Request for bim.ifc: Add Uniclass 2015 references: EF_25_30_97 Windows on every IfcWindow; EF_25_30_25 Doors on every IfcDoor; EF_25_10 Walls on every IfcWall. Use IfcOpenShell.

First a look at what the model holds.

```python
import ifcopenshell

model = ifcopenshell.open("bim.ifc")
print(model.schema)
print("classifications:", [c.Name for c in model.by_type("IfcClassification")])
for ifc_class in ("IfcDoor", "IfcRoof", "IfcStair", "IfcWall", "IfcWindow"):
    print(ifc_class, len(model.by_type(ifc_class)))
```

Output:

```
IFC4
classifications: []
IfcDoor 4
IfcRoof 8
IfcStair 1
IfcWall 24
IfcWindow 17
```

```python
import ifcopenshell
import ifcopenshell.api.classification

model = ifcopenshell.open("bim.ifc")

system = ifcopenshell.api.classification.add_classification(model, classification="Uniclass 2015")

codes = {
    "IfcWindow": ("EF_25_30_97", "Windows"),
    "IfcDoor": ("EF_25_30_25", "Doors"),
    "IfcWall": ("EF_25_10", "Walls"),
}
for ifc_class, (code, name) in codes.items():
    products = model.by_type(ifc_class)
    ifcopenshell.api.classification.add_reference(
        model, products=products, classification=system, identification=code, name=name
    )
    print(code, len(products))

model.write("bim_updated.ifc")
```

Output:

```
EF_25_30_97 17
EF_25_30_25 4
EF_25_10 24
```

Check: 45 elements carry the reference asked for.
